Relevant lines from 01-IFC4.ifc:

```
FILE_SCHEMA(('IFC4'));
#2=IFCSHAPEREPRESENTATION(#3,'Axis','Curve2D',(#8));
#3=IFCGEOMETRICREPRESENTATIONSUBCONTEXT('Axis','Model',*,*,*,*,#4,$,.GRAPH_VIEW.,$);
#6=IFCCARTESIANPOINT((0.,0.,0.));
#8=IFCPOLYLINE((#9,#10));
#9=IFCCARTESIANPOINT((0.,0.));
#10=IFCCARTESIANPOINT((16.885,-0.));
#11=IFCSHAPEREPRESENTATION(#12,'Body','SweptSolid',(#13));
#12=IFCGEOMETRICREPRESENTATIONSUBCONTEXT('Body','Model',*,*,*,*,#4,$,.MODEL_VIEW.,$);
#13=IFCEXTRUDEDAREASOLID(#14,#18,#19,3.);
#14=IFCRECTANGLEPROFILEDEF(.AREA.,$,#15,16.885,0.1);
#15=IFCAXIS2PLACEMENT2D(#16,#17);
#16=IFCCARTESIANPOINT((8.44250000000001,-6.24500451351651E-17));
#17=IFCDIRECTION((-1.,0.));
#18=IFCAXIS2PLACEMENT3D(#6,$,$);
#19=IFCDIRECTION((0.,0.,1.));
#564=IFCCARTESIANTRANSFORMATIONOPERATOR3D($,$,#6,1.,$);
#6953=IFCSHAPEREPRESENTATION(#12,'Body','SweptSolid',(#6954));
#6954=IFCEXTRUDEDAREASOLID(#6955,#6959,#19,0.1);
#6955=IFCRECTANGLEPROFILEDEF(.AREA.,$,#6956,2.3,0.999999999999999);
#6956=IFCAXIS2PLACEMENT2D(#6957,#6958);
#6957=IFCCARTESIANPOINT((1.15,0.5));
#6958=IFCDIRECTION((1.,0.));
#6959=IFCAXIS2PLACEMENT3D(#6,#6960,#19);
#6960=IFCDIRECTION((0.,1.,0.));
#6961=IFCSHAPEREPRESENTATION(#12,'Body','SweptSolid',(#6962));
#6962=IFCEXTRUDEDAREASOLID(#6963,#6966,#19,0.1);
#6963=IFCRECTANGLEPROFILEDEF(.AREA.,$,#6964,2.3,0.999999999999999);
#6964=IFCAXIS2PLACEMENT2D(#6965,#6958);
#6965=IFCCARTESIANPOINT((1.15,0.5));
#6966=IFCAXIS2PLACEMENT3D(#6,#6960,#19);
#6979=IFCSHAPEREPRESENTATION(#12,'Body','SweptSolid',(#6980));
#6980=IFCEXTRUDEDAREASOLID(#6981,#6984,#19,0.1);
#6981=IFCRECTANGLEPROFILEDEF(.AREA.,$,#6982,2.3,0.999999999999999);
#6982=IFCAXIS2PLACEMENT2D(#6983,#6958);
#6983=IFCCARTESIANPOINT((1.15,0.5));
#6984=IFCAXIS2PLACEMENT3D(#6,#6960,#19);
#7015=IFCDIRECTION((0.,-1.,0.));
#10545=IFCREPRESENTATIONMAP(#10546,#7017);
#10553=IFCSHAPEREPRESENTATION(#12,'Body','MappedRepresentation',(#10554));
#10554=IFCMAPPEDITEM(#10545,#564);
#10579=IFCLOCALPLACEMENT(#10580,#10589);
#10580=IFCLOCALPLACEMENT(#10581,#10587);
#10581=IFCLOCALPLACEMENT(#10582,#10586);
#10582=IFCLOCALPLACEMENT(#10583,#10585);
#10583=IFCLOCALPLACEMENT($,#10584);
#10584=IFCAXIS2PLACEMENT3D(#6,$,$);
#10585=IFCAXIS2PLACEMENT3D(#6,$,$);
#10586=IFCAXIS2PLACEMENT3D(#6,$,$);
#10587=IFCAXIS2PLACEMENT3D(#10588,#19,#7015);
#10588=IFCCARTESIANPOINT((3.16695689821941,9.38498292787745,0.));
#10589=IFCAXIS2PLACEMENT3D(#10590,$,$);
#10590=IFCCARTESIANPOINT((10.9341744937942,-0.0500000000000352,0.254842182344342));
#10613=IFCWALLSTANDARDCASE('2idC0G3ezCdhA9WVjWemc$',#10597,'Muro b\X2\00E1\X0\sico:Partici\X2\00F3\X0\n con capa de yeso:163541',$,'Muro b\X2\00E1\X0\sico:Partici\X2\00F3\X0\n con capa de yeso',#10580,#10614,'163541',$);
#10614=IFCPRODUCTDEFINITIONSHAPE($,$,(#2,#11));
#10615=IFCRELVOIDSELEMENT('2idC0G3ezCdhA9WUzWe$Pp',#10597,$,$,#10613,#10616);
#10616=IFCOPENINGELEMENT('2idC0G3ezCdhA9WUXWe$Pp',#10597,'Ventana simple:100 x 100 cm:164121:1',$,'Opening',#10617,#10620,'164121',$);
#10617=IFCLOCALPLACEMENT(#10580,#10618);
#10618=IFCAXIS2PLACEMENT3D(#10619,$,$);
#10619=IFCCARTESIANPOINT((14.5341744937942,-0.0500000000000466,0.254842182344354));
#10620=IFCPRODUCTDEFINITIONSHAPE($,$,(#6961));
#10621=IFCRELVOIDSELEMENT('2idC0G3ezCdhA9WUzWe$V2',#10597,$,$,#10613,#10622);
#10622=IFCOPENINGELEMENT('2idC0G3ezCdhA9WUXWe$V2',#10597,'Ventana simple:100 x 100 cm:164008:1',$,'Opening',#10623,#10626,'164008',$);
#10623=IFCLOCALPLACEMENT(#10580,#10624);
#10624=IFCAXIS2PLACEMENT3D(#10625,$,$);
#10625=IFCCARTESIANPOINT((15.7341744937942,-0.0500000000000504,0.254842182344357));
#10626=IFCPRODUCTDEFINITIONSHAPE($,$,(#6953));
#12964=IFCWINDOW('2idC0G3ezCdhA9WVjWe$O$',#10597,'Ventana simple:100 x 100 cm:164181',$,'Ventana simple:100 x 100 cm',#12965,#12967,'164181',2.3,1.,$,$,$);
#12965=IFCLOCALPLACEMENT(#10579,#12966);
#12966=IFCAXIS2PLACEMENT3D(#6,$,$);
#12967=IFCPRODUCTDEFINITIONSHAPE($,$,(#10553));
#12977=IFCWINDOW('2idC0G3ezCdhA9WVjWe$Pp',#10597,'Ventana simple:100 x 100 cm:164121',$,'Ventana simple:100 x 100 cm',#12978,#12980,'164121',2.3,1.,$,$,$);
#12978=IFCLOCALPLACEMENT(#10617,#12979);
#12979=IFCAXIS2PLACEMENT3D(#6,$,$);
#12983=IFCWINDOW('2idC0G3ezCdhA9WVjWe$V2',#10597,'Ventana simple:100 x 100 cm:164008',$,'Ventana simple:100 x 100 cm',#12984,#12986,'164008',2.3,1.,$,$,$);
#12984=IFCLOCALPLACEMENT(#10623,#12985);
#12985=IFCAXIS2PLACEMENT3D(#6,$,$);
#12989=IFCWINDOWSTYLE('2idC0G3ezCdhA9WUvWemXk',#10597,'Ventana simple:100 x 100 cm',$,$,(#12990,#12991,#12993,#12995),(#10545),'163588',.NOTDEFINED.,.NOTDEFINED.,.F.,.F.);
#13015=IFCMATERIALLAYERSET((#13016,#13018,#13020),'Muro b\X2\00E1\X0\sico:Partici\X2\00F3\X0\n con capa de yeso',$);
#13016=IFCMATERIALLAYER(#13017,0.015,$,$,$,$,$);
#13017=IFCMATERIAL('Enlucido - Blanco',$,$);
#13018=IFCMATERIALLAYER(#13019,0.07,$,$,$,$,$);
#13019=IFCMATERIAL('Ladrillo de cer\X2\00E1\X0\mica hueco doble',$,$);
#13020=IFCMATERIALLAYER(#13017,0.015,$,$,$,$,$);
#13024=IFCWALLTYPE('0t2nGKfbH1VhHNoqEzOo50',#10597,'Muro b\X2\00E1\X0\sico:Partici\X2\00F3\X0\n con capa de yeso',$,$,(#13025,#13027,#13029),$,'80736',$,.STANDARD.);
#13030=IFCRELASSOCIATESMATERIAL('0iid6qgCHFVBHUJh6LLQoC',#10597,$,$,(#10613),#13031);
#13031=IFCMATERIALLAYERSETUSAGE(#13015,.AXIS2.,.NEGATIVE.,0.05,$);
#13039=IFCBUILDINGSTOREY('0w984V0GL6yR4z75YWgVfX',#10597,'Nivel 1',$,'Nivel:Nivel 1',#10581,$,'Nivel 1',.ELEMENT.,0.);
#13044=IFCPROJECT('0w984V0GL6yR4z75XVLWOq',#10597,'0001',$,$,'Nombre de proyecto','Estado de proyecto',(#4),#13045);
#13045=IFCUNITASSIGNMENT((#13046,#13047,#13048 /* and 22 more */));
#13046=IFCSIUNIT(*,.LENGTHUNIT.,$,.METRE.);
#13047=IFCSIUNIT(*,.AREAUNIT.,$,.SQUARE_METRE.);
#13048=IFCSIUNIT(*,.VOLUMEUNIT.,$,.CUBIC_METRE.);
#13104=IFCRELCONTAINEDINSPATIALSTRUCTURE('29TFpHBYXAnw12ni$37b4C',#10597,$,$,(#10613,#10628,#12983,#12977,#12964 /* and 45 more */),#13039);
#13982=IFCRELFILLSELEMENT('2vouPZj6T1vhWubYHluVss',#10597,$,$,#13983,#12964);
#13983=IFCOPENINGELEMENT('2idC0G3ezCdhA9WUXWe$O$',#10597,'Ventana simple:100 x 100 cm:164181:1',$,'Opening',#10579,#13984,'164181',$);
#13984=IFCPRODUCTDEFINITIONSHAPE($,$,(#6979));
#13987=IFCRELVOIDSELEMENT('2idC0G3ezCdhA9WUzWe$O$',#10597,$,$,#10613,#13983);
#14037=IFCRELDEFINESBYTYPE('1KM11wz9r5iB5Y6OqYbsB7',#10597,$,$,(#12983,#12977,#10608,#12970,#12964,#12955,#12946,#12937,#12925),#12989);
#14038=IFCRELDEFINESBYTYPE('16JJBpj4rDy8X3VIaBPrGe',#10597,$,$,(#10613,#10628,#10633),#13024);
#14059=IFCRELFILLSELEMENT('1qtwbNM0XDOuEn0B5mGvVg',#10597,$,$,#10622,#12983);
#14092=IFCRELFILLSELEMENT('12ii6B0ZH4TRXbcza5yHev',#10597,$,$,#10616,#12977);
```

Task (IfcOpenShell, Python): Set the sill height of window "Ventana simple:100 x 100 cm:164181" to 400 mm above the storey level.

```python
import numpy as np
import ifcopenshell
import ifcopenshell.api.geometry
import ifcopenshell.geom
import ifcopenshell.util.element
import ifcopenshell.util.placement
import ifcopenshell.util.shape
import ifcopenshell.util.unit

model = ifcopenshell.open("01-IFC4.ifc")
unit_scale = ifcopenshell.util.unit.calculate_unit_scale(model)

window = model.by_id(12964)
opening = window.FillsVoids[0].RelatingOpeningElement
storey = ifcopenshell.util.element.get_container(window, ifc_class="IfcBuildingStorey")
level = ifcopenshell.util.placement.get_local_placement(storey.ObjectPlacement)[2, 3]

# The opening's origin need not be at the sill, so measure its lowest point.
shape = ifcopenshell.geom.create_shape(ifcopenshell.geom.settings(), opening)
bottom = ifcopenshell.util.shape.get_shape_bottom_elevation(shape, shape.geometry) / unit_scale
dz = level + 0.4 / unit_scale - bottom

shift = np.array([0.0, 0.0, dz])
# The window is placed relative to its opening, so it follows when the opening moves.
matrix = ifcopenshell.util.placement.get_local_placement(opening.ObjectPlacement)
matrix[:3, 3] += shift
ifcopenshell.api.geometry.edit_object_placement(
    model, product=opening, matrix=matrix, is_si=False, should_transform_children=True
)

print(f"moved by {dz * unit_scale:+.3f} m")

model.write("01-IFC4_updated.ifc")
```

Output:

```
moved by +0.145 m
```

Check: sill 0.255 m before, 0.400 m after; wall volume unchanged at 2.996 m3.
